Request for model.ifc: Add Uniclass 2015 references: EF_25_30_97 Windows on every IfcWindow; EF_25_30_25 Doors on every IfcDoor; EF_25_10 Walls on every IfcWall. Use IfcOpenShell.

First a look at what the model holds.

```python
import ifcopenshell

model = ifcopenshell.open("model.ifc")
print(model.schema)
print("classifications:", [c.Name for c in model.by_type("IfcClassification")])
for ifc_class in ("IfcDoor", "IfcRoof", "IfcStair", "IfcWall", "IfcWindow"):
    print(ifc_class, len(model.by_type(ifc_class)))
```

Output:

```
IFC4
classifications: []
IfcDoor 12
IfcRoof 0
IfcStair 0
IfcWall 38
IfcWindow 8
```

```python
import ifcopenshell
import ifcopenshell.api.classification

model = ifcopenshell.open("model.ifc")

system = ifcopenshell.api.classification.add_classification(model, classification="Uniclass 2015")

codes = {
    "IfcWindow": ("EF_25_30_97", "Windows"),
    "IfcDoor": ("EF_25_30_25", "Doors"),
    "IfcWall": ("EF_25_10", "Walls"),
}
for ifc_class, (code, name) in codes.items():
    products = model.by_type(ifc_class)
    ifcopenshell.api.classification.add_reference(
        model, products=products, classification=system, identification=code, name=name
    )
    print(code, len(products))

model.write("model_edited.ifc")
```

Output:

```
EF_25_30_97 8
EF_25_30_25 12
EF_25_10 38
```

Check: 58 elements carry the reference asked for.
